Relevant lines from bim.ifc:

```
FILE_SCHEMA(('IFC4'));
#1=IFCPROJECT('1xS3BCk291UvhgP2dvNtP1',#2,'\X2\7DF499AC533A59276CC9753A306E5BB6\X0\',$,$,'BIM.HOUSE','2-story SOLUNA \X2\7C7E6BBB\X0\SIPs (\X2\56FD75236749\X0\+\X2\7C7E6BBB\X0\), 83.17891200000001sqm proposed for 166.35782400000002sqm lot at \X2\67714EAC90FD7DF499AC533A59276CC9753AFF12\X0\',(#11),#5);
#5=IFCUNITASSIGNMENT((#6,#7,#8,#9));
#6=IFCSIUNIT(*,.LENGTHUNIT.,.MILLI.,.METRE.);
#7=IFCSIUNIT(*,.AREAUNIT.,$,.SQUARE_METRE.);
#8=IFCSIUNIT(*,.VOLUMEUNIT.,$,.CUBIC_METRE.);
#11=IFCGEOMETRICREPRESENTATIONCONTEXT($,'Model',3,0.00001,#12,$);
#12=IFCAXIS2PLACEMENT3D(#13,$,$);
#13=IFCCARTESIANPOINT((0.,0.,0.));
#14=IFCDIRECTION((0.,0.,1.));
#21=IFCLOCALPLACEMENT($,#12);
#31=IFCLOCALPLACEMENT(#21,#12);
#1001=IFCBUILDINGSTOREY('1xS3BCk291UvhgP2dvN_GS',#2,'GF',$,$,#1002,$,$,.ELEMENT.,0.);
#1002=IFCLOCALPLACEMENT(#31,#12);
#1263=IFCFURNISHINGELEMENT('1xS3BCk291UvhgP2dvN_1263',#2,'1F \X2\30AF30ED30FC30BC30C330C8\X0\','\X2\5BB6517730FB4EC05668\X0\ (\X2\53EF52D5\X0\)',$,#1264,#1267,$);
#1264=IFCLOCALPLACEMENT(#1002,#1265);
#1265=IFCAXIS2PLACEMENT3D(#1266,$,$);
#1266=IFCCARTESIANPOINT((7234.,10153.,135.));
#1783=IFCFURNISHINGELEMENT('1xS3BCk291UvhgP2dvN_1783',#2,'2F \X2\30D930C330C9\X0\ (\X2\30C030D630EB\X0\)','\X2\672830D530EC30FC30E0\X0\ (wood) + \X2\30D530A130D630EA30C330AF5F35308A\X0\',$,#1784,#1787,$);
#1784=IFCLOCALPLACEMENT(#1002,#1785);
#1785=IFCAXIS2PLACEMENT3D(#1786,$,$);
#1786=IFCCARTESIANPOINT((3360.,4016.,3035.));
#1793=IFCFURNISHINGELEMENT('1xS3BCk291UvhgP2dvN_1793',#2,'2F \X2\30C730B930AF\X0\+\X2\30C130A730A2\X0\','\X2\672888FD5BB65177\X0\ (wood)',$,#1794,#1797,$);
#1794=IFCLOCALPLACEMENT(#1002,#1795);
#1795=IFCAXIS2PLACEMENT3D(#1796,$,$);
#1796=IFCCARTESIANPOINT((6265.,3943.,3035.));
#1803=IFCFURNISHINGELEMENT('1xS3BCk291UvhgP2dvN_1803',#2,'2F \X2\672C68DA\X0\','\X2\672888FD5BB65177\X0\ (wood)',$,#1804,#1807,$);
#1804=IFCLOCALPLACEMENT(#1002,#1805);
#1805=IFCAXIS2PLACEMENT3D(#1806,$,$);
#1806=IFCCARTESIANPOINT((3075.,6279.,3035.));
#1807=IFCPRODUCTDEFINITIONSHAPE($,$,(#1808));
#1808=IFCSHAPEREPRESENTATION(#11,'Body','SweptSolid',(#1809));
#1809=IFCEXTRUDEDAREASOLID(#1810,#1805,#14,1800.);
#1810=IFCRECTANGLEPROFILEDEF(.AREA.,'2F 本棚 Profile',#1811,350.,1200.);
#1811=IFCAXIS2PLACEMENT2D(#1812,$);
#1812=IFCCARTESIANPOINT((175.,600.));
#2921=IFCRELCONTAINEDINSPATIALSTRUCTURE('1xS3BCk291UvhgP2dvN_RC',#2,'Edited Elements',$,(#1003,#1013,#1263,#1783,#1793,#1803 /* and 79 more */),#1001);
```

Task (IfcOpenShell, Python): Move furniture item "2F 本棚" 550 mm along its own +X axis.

```python
import ifcopenshell
import ifcopenshell.api.geometry
import ifcopenshell.util.placement

model = ifcopenshell.open("bim.ifc")

item = model.by_guid("1xS3BCk291UvhgP2dvN_1803")
matrix = ifcopenshell.util.placement.get_local_placement(item.ObjectPlacement)
matrix[:3, 3] += matrix[:3, 0] * 550.0
ifcopenshell.api.geometry.edit_object_placement(model, product=item, matrix=matrix, is_si=False)

print(ifcopenshell.util.placement.get_local_placement(item.ObjectPlacement).round(3) + 0.0)

model.write("bim-out.ifc")
```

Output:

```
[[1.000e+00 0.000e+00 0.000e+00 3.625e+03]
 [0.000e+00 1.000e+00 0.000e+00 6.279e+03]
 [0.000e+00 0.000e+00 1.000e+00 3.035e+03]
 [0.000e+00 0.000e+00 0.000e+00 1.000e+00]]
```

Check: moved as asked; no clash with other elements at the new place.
